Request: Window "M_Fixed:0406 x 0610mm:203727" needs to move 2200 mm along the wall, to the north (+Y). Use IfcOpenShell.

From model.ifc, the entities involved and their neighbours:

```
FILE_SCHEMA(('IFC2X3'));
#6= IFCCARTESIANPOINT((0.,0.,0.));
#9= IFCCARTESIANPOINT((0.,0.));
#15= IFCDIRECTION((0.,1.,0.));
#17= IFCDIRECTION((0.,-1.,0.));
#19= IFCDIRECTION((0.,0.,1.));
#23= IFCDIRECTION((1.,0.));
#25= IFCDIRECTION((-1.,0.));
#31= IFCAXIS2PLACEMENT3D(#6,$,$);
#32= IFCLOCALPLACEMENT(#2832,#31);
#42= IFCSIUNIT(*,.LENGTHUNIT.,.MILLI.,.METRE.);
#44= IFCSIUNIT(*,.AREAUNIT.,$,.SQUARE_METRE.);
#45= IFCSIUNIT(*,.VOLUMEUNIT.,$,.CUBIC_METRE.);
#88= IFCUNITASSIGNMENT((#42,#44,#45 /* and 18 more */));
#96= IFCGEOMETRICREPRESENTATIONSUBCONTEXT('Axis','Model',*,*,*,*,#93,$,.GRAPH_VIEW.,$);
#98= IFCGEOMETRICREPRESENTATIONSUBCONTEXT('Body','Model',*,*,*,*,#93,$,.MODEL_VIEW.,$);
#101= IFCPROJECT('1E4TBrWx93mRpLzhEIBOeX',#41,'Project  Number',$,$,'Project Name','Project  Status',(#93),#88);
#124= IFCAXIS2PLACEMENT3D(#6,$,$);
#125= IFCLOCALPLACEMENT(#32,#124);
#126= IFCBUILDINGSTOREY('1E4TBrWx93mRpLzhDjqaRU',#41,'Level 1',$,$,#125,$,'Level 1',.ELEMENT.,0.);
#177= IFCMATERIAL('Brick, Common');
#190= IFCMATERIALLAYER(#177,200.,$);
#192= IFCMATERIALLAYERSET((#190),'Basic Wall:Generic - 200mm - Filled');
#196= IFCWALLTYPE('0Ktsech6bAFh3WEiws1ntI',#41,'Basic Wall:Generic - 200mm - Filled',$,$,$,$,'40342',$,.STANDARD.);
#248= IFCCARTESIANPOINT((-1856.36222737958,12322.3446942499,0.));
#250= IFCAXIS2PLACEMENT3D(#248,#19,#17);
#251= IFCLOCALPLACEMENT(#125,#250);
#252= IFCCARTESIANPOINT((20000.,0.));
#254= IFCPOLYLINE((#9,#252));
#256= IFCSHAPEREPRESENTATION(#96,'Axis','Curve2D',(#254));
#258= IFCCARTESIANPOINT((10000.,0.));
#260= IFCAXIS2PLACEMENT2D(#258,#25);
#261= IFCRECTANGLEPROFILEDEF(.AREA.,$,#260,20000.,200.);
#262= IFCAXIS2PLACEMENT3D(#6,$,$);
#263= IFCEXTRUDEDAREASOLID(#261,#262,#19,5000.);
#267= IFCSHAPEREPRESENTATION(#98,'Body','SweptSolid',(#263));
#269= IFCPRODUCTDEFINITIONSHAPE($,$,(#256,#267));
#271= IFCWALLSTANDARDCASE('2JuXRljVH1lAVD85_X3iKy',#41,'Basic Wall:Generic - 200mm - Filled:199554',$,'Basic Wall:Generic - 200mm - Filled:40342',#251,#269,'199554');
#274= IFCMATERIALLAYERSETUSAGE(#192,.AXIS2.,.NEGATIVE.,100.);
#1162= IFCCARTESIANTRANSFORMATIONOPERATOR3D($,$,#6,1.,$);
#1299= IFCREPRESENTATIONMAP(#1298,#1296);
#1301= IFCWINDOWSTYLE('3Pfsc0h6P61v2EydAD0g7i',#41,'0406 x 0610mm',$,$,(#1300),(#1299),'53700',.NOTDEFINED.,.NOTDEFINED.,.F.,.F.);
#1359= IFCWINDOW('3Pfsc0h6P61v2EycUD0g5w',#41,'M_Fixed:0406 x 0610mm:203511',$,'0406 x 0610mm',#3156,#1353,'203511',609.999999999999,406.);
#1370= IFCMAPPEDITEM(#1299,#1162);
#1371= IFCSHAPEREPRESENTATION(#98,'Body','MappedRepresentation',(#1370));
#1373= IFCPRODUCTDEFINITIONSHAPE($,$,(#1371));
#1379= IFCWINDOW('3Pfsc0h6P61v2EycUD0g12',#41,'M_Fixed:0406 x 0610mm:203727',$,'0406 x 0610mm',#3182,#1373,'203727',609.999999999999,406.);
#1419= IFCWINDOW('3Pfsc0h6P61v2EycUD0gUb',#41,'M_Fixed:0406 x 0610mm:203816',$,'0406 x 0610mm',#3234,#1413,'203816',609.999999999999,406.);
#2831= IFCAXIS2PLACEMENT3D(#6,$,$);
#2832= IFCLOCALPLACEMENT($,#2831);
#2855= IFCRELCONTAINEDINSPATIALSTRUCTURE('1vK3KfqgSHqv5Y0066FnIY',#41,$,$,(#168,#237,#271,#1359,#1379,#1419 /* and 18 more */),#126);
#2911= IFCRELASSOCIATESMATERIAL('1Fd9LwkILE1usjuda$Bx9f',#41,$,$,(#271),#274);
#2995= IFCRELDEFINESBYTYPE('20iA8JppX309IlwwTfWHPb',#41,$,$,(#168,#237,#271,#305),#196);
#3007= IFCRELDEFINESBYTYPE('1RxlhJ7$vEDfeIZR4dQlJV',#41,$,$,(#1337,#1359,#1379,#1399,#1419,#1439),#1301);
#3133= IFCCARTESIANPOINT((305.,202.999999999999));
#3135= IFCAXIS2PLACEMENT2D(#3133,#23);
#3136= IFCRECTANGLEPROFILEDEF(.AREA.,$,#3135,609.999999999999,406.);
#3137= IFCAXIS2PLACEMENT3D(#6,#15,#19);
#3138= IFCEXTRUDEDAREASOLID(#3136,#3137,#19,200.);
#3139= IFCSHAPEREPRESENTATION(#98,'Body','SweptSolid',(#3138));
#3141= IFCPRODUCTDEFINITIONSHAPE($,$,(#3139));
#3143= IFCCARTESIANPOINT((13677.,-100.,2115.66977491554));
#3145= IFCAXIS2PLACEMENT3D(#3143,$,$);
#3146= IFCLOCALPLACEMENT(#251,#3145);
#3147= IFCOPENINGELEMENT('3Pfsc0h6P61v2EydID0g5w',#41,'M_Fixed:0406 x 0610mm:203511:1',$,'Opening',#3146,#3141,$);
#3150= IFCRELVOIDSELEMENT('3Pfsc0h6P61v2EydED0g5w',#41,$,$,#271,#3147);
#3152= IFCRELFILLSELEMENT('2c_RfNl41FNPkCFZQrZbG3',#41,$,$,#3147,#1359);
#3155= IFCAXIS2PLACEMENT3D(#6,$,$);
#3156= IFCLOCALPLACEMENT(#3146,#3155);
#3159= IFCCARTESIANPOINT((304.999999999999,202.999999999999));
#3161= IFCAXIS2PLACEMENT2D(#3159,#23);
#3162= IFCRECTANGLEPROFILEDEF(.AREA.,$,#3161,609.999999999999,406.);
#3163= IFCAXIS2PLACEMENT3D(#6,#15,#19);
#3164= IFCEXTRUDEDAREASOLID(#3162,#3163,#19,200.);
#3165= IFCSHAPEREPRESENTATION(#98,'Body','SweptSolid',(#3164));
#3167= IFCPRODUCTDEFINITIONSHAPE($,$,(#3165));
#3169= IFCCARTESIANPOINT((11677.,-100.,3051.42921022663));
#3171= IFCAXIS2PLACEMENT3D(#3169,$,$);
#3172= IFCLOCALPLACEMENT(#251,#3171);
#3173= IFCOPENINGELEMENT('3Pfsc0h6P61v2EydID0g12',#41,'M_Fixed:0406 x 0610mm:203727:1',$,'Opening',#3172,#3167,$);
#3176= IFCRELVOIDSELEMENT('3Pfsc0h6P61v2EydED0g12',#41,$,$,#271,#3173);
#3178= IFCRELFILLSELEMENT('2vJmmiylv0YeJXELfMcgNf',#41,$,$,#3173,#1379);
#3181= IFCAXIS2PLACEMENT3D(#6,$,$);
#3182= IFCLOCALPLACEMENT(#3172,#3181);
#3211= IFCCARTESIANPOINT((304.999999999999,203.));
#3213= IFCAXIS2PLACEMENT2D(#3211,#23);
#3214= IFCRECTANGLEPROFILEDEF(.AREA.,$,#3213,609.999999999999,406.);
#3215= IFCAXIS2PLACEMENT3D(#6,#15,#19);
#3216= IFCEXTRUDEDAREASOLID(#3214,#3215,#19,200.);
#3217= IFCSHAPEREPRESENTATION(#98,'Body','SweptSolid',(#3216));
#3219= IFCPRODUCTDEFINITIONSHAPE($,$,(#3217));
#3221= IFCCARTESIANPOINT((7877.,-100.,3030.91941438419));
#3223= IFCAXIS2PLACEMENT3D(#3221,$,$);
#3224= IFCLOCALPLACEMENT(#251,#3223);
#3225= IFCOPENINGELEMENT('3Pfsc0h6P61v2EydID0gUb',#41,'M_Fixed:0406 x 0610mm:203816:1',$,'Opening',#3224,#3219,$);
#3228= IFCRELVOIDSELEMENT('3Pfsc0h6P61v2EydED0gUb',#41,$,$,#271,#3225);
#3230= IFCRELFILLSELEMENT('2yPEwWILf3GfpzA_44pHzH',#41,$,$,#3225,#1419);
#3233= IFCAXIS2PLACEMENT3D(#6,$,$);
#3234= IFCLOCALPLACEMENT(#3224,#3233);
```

```python
import ifcopenshell
import ifcopenshell.api.geometry
import ifcopenshell.util.placement

model = ifcopenshell.open("model.ifc")

window = model.by_id(1379)
opening = window.FillsVoids[0].RelatingOpeningElement
wall = opening.VoidsElements[0].RelatingBuildingElement

wall_matrix = ifcopenshell.util.placement.get_local_placement(wall.ObjectPlacement)
shift = wall_matrix[:3, 0] * -2200.0
before = ifcopenshell.util.placement.get_local_placement(window.ObjectPlacement)[:3, 3].copy()

# The window is placed relative to its opening, so it follows when the opening moves.
matrix = ifcopenshell.util.placement.get_local_placement(opening.ObjectPlacement)
matrix[:3, 3] += shift
ifcopenshell.api.geometry.edit_object_placement(
    model, product=opening, matrix=matrix, is_si=False, should_transform_children=True
)

after = ifcopenshell.util.placement.get_local_placement(window.ObjectPlacement)[:3, 3]
print("window moved by", (after - before).round(3) + 0.0)

model.write("model_rev.ifc")
```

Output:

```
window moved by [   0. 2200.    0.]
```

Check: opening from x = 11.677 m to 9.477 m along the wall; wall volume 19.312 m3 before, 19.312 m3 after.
